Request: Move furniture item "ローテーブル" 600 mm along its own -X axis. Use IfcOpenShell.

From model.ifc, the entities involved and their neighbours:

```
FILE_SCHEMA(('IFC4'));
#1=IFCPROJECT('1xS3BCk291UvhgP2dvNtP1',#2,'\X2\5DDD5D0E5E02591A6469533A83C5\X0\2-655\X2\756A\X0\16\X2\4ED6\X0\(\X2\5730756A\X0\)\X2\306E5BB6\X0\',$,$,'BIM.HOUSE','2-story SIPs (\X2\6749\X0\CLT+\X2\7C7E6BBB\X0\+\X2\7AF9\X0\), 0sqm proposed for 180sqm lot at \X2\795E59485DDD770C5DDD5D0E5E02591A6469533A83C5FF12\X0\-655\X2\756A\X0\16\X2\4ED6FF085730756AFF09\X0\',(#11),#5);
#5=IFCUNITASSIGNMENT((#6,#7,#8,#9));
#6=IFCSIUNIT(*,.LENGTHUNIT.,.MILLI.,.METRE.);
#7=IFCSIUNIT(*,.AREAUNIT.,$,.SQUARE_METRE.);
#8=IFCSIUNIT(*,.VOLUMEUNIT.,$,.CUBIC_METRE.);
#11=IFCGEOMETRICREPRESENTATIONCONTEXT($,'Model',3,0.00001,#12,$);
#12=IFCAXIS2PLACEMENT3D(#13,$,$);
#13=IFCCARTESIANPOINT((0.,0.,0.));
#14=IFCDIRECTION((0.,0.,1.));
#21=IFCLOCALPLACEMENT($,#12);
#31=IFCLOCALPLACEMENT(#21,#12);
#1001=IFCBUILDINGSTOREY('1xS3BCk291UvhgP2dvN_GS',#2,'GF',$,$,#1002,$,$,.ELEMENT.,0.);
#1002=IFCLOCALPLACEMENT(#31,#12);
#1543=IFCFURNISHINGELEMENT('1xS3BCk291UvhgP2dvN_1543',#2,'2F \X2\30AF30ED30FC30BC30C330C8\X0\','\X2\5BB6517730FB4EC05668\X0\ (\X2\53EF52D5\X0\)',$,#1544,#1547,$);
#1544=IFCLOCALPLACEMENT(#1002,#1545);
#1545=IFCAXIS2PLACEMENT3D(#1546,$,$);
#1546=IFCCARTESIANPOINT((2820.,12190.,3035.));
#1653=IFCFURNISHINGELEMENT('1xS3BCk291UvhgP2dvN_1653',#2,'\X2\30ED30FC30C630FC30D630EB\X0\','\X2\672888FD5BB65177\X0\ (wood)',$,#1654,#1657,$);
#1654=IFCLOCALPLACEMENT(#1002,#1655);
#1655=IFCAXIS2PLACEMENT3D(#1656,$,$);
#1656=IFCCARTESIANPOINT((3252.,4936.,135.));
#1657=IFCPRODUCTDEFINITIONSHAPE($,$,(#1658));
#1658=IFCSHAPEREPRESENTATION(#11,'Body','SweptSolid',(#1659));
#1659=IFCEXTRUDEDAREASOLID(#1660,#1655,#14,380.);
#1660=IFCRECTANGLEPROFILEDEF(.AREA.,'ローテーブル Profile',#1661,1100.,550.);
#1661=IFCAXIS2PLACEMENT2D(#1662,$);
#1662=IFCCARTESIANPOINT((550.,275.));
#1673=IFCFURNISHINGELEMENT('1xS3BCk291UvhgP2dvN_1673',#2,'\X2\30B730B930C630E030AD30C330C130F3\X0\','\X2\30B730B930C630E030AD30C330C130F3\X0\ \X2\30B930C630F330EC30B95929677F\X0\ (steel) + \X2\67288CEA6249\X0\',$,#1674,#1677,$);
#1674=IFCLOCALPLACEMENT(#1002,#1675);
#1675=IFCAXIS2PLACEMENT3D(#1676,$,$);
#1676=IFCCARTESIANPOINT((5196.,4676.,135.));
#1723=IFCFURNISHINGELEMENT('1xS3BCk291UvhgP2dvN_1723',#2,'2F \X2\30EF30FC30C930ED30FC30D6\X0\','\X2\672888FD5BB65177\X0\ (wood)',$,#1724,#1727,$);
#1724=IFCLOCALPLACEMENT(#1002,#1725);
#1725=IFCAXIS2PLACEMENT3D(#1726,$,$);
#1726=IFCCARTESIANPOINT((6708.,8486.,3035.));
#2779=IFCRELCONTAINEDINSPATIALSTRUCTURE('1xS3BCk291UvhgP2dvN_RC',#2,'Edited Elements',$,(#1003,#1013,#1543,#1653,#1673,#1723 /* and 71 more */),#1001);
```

```python
import ifcopenshell
import ifcopenshell.api.geometry
import ifcopenshell.util.placement
import ifcopenshell.util.unit

model = ifcopenshell.open("model.ifc")
unit_scale = ifcopenshell.util.unit.calculate_unit_scale(model)

item = model.by_guid("1xS3BCk291UvhgP2dvN_1653")
matrix = ifcopenshell.util.placement.get_local_placement(item.ObjectPlacement)
matrix[:3, 3] -= matrix[:3, 0] * 0.6 / unit_scale
ifcopenshell.api.geometry.edit_object_placement(model, product=item, matrix=matrix, is_si=False)

print(ifcopenshell.util.placement.get_local_placement(item.ObjectPlacement).round(3) + 0.0)

model.write("model_v2.ifc")
```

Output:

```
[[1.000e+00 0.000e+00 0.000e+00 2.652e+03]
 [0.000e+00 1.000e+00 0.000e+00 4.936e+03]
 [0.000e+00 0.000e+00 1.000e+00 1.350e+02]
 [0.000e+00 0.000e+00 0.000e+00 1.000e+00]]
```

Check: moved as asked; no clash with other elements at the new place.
